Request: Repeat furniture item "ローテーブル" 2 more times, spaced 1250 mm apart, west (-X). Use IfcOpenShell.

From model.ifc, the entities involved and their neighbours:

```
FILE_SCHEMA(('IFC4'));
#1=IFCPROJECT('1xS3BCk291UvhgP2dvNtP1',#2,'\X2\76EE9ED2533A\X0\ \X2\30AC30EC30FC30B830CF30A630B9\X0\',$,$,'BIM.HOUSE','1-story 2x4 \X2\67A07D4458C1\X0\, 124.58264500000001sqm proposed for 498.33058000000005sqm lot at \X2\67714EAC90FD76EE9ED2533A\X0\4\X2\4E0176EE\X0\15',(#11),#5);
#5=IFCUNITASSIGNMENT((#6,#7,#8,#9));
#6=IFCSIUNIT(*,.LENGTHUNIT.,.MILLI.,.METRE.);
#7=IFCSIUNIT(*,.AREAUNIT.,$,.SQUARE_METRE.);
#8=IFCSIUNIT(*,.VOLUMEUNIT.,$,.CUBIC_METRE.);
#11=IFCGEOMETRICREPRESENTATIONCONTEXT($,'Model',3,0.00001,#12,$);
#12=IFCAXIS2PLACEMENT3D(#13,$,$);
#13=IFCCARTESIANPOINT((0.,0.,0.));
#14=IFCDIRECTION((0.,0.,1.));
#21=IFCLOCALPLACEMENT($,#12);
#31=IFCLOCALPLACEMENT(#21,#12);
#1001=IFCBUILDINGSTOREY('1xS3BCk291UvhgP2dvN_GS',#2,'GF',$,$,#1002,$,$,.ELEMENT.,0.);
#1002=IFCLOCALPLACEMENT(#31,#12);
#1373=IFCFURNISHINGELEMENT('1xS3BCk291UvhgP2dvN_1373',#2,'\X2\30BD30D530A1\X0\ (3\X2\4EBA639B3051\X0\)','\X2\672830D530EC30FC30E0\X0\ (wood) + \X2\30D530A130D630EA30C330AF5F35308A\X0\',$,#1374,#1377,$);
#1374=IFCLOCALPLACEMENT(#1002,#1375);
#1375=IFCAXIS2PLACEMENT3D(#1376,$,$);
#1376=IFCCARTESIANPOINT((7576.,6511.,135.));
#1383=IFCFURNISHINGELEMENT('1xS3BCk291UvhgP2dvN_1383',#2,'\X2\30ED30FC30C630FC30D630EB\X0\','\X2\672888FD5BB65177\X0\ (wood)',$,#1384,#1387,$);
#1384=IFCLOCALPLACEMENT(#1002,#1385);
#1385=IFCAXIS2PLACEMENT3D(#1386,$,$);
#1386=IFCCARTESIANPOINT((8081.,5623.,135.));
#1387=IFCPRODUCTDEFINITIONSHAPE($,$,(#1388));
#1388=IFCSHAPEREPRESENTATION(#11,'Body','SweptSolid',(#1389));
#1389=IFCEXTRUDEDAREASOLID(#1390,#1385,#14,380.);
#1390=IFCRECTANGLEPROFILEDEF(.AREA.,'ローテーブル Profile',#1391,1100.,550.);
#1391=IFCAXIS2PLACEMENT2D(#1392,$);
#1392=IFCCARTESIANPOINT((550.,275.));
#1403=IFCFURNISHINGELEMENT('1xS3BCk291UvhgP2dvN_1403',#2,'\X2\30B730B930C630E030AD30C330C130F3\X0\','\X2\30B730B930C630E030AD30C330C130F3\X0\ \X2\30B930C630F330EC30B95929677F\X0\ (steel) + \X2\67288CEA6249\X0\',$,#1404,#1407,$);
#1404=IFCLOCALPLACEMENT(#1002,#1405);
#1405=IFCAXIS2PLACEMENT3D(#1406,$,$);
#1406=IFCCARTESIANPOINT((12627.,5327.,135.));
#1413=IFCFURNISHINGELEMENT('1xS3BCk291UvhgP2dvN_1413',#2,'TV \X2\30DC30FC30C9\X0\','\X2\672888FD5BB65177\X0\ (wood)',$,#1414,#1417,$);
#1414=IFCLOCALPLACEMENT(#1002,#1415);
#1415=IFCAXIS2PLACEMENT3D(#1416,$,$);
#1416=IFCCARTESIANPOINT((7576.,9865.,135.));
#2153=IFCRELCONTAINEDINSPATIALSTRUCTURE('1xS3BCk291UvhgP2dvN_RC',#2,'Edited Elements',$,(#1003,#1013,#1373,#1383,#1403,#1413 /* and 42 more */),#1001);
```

```python
import numpy as np
import ifcopenshell
import ifcopenshell.api.geometry
import ifcopenshell.api.root
import ifcopenshell.util.element
import ifcopenshell.util.placement

model = ifcopenshell.open("model.ifc")


def reuse_history(source, copy):
    """copy_class also copies each property set's owner history, people and application; keep the originals."""
    for rel in copy.IsDefinedBy:
        if rel.is_a("IfcRelDefinesByProperties") and (history := rel.RelatingPropertyDefinition.OwnerHistory):
            rel.RelatingPropertyDefinition.OwnerHistory = source.OwnerHistory
            ifcopenshell.util.element.remove_deep2(model, history)


source = model.by_guid("1xS3BCk291UvhgP2dvN_1383")
base = ifcopenshell.util.placement.get_local_placement(source.ObjectPlacement)
step = np.array([-1.0, 0.0, 0.0]) * 1250.0

for i in range(1, 3):
    copy = ifcopenshell.api.root.copy_class(model, product=source)
    copy.Representation = ifcopenshell.util.element.copy_deep(
        model, source.Representation, exclude=["IfcGeometricRepresentationContext", "IfcRepresentationMap"]
    )
    reuse_history(source, copy)
    matrix = base.copy()
    matrix[:3, 3] += i * step
    print("added at", matrix[:3, 3].round(3) + 0.0)
    ifcopenshell.api.geometry.edit_object_placement(model, product=copy, matrix=matrix, is_si=False)

model.write("model_updated.ifc")
```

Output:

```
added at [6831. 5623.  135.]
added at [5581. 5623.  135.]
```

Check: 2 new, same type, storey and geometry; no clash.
